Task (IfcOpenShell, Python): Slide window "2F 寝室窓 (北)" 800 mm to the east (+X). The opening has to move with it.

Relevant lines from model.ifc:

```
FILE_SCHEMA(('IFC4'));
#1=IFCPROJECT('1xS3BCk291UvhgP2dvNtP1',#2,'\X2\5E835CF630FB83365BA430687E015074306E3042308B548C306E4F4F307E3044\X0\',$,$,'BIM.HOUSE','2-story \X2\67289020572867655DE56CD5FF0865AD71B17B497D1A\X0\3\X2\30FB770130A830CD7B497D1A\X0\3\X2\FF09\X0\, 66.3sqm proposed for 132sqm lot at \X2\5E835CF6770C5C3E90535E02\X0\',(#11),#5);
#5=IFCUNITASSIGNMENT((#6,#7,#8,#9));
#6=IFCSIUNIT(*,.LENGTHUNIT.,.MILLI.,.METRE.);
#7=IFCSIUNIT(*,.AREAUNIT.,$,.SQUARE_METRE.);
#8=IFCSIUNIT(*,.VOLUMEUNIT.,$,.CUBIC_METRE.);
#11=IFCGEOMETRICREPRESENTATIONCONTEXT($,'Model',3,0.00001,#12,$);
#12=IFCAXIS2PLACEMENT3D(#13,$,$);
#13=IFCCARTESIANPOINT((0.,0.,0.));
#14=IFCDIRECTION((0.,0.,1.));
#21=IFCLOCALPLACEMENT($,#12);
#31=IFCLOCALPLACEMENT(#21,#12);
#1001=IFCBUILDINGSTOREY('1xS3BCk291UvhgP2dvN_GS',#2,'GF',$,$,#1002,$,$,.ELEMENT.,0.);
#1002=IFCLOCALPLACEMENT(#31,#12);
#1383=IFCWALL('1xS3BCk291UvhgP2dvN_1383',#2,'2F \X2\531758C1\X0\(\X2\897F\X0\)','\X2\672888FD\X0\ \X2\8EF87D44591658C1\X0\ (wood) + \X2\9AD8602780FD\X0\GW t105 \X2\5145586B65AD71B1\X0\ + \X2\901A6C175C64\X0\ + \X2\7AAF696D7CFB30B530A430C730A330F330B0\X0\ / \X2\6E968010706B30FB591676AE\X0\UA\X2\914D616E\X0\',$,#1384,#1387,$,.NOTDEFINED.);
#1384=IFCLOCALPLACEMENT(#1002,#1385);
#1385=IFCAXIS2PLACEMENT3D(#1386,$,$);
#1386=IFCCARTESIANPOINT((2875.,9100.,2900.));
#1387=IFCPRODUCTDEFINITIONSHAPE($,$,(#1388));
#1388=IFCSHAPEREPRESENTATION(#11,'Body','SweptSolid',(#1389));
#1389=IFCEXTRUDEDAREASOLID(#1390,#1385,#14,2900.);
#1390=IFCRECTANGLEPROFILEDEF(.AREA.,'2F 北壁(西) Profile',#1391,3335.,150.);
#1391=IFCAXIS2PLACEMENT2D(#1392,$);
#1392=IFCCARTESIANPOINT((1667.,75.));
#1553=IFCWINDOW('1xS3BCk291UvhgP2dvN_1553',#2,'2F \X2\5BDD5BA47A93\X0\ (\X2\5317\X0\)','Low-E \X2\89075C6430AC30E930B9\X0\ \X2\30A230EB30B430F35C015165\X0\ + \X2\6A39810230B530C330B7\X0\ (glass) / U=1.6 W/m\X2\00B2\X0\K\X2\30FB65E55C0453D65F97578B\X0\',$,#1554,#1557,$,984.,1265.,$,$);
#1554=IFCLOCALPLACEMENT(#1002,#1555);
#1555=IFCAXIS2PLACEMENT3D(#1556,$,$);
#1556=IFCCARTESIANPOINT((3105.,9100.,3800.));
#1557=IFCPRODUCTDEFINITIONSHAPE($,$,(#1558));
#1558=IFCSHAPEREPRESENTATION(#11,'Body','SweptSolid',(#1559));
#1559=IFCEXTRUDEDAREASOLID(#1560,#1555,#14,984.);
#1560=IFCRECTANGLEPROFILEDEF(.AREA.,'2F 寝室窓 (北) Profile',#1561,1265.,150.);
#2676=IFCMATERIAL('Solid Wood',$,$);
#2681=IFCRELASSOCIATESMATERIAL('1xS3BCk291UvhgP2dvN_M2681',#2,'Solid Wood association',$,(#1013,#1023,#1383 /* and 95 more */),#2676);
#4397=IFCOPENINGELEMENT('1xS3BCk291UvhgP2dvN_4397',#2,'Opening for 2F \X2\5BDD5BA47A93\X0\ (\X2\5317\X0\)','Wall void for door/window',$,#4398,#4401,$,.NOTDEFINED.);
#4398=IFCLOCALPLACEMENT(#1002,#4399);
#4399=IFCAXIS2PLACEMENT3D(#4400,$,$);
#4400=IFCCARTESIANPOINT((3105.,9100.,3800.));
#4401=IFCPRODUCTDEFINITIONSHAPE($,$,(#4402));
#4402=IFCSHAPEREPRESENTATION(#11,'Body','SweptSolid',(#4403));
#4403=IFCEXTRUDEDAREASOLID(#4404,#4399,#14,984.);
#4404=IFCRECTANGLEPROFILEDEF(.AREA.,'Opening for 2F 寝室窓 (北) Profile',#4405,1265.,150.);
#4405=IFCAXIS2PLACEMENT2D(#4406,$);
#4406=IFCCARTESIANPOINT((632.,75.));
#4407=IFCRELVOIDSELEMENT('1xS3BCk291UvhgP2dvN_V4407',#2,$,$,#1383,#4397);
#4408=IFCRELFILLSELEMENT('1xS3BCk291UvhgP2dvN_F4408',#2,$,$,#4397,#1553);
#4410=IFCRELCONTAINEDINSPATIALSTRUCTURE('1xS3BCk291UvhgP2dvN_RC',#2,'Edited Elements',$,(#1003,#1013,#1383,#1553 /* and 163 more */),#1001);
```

```python
import ifcopenshell
import ifcopenshell.api.geometry
import ifcopenshell.util.placement

model = ifcopenshell.open("model.ifc")

window = model.by_guid("1xS3BCk291UvhgP2dvN_1553")
opening = window.FillsVoids[0].RelatingOpeningElement
wall = opening.VoidsElements[0].RelatingBuildingElement

wall_matrix = ifcopenshell.util.placement.get_local_placement(wall.ObjectPlacement)
shift = wall_matrix[:3, 0] * 800.0
before = ifcopenshell.util.placement.get_local_placement(window.ObjectPlacement)[:3, 3].copy()

# The window is not placed relative to its opening, so move both.
for product in (opening, window):
    matrix = ifcopenshell.util.placement.get_local_placement(product.ObjectPlacement)
    matrix[:3, 3] += shift
    ifcopenshell.api.geometry.edit_object_placement(model, product=product, matrix=matrix, is_si=False)

after = ifcopenshell.util.placement.get_local_placement(window.ObjectPlacement)[:3, 3]
print("window moved by", (after - before).round(3) + 0.0)

model.write("model_updated.ifc")
```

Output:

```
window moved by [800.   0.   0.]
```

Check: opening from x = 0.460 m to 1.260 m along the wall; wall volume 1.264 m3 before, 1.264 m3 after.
